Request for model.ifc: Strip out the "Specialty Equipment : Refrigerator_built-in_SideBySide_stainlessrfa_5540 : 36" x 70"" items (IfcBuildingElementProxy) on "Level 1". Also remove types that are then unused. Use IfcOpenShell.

First a look at what the model holds.

```python
import ifcopenshell
import ifcopenshell.util.element

model = ifcopenshell.open("model.ifc")
print(model.schema)
storey = next(s for s in model.by_type("IfcBuildingStorey") if s.Name == "Level 1")
proxies = [e for e in ifcopenshell.util.element.get_decomposition(storey) if e.is_a("IfcBuildingElementProxy")]
seen = {}
for e in proxies:
    element_type = ifcopenshell.util.element.get_type(e)
    name = element_type.Name if element_type not in (None, e) else None
    seen[name] = seen.get(name, 0) + 1
for name, count in sorted(seen.items(), key=str):
    print(count, "x", name)
```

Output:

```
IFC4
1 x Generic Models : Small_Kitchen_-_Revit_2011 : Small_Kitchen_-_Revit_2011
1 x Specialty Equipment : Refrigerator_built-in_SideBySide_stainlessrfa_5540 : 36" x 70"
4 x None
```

```python
import ifcopenshell
import ifcopenshell.api.root
import ifcopenshell.util.element

model = ifcopenshell.open("model.ifc")

storey = next(s for s in model.by_type("IfcBuildingStorey") if s.Name == "Level 1")
proxies = [e for e in ifcopenshell.util.element.get_decomposition(storey) if e.is_a("IfcBuildingElementProxy")]
targets = [e for e in proxies if (t := ifcopenshell.util.element.get_type(e)) not in (None, e) and t.Name == 'Specialty Equipment : Refrigerator_built-in_SideBySide_stainlessrfa_5540 : 36" x 70"']
types = {ifcopenshell.util.element.get_type(e) for e in targets} - {None, *targets}

for e in targets:
    ifcopenshell.api.root.remove_product(model, product=e)
print(len(targets), "removed")

unused = [t for t in types if not ifcopenshell.util.element.get_types(t)]
for t in unused:
    ifcopenshell.api.root.remove_product(model, product=t)
print(len(unused), "unused types removed")

model.write("model_rev.ifc")
```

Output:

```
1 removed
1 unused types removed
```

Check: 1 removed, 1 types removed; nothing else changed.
